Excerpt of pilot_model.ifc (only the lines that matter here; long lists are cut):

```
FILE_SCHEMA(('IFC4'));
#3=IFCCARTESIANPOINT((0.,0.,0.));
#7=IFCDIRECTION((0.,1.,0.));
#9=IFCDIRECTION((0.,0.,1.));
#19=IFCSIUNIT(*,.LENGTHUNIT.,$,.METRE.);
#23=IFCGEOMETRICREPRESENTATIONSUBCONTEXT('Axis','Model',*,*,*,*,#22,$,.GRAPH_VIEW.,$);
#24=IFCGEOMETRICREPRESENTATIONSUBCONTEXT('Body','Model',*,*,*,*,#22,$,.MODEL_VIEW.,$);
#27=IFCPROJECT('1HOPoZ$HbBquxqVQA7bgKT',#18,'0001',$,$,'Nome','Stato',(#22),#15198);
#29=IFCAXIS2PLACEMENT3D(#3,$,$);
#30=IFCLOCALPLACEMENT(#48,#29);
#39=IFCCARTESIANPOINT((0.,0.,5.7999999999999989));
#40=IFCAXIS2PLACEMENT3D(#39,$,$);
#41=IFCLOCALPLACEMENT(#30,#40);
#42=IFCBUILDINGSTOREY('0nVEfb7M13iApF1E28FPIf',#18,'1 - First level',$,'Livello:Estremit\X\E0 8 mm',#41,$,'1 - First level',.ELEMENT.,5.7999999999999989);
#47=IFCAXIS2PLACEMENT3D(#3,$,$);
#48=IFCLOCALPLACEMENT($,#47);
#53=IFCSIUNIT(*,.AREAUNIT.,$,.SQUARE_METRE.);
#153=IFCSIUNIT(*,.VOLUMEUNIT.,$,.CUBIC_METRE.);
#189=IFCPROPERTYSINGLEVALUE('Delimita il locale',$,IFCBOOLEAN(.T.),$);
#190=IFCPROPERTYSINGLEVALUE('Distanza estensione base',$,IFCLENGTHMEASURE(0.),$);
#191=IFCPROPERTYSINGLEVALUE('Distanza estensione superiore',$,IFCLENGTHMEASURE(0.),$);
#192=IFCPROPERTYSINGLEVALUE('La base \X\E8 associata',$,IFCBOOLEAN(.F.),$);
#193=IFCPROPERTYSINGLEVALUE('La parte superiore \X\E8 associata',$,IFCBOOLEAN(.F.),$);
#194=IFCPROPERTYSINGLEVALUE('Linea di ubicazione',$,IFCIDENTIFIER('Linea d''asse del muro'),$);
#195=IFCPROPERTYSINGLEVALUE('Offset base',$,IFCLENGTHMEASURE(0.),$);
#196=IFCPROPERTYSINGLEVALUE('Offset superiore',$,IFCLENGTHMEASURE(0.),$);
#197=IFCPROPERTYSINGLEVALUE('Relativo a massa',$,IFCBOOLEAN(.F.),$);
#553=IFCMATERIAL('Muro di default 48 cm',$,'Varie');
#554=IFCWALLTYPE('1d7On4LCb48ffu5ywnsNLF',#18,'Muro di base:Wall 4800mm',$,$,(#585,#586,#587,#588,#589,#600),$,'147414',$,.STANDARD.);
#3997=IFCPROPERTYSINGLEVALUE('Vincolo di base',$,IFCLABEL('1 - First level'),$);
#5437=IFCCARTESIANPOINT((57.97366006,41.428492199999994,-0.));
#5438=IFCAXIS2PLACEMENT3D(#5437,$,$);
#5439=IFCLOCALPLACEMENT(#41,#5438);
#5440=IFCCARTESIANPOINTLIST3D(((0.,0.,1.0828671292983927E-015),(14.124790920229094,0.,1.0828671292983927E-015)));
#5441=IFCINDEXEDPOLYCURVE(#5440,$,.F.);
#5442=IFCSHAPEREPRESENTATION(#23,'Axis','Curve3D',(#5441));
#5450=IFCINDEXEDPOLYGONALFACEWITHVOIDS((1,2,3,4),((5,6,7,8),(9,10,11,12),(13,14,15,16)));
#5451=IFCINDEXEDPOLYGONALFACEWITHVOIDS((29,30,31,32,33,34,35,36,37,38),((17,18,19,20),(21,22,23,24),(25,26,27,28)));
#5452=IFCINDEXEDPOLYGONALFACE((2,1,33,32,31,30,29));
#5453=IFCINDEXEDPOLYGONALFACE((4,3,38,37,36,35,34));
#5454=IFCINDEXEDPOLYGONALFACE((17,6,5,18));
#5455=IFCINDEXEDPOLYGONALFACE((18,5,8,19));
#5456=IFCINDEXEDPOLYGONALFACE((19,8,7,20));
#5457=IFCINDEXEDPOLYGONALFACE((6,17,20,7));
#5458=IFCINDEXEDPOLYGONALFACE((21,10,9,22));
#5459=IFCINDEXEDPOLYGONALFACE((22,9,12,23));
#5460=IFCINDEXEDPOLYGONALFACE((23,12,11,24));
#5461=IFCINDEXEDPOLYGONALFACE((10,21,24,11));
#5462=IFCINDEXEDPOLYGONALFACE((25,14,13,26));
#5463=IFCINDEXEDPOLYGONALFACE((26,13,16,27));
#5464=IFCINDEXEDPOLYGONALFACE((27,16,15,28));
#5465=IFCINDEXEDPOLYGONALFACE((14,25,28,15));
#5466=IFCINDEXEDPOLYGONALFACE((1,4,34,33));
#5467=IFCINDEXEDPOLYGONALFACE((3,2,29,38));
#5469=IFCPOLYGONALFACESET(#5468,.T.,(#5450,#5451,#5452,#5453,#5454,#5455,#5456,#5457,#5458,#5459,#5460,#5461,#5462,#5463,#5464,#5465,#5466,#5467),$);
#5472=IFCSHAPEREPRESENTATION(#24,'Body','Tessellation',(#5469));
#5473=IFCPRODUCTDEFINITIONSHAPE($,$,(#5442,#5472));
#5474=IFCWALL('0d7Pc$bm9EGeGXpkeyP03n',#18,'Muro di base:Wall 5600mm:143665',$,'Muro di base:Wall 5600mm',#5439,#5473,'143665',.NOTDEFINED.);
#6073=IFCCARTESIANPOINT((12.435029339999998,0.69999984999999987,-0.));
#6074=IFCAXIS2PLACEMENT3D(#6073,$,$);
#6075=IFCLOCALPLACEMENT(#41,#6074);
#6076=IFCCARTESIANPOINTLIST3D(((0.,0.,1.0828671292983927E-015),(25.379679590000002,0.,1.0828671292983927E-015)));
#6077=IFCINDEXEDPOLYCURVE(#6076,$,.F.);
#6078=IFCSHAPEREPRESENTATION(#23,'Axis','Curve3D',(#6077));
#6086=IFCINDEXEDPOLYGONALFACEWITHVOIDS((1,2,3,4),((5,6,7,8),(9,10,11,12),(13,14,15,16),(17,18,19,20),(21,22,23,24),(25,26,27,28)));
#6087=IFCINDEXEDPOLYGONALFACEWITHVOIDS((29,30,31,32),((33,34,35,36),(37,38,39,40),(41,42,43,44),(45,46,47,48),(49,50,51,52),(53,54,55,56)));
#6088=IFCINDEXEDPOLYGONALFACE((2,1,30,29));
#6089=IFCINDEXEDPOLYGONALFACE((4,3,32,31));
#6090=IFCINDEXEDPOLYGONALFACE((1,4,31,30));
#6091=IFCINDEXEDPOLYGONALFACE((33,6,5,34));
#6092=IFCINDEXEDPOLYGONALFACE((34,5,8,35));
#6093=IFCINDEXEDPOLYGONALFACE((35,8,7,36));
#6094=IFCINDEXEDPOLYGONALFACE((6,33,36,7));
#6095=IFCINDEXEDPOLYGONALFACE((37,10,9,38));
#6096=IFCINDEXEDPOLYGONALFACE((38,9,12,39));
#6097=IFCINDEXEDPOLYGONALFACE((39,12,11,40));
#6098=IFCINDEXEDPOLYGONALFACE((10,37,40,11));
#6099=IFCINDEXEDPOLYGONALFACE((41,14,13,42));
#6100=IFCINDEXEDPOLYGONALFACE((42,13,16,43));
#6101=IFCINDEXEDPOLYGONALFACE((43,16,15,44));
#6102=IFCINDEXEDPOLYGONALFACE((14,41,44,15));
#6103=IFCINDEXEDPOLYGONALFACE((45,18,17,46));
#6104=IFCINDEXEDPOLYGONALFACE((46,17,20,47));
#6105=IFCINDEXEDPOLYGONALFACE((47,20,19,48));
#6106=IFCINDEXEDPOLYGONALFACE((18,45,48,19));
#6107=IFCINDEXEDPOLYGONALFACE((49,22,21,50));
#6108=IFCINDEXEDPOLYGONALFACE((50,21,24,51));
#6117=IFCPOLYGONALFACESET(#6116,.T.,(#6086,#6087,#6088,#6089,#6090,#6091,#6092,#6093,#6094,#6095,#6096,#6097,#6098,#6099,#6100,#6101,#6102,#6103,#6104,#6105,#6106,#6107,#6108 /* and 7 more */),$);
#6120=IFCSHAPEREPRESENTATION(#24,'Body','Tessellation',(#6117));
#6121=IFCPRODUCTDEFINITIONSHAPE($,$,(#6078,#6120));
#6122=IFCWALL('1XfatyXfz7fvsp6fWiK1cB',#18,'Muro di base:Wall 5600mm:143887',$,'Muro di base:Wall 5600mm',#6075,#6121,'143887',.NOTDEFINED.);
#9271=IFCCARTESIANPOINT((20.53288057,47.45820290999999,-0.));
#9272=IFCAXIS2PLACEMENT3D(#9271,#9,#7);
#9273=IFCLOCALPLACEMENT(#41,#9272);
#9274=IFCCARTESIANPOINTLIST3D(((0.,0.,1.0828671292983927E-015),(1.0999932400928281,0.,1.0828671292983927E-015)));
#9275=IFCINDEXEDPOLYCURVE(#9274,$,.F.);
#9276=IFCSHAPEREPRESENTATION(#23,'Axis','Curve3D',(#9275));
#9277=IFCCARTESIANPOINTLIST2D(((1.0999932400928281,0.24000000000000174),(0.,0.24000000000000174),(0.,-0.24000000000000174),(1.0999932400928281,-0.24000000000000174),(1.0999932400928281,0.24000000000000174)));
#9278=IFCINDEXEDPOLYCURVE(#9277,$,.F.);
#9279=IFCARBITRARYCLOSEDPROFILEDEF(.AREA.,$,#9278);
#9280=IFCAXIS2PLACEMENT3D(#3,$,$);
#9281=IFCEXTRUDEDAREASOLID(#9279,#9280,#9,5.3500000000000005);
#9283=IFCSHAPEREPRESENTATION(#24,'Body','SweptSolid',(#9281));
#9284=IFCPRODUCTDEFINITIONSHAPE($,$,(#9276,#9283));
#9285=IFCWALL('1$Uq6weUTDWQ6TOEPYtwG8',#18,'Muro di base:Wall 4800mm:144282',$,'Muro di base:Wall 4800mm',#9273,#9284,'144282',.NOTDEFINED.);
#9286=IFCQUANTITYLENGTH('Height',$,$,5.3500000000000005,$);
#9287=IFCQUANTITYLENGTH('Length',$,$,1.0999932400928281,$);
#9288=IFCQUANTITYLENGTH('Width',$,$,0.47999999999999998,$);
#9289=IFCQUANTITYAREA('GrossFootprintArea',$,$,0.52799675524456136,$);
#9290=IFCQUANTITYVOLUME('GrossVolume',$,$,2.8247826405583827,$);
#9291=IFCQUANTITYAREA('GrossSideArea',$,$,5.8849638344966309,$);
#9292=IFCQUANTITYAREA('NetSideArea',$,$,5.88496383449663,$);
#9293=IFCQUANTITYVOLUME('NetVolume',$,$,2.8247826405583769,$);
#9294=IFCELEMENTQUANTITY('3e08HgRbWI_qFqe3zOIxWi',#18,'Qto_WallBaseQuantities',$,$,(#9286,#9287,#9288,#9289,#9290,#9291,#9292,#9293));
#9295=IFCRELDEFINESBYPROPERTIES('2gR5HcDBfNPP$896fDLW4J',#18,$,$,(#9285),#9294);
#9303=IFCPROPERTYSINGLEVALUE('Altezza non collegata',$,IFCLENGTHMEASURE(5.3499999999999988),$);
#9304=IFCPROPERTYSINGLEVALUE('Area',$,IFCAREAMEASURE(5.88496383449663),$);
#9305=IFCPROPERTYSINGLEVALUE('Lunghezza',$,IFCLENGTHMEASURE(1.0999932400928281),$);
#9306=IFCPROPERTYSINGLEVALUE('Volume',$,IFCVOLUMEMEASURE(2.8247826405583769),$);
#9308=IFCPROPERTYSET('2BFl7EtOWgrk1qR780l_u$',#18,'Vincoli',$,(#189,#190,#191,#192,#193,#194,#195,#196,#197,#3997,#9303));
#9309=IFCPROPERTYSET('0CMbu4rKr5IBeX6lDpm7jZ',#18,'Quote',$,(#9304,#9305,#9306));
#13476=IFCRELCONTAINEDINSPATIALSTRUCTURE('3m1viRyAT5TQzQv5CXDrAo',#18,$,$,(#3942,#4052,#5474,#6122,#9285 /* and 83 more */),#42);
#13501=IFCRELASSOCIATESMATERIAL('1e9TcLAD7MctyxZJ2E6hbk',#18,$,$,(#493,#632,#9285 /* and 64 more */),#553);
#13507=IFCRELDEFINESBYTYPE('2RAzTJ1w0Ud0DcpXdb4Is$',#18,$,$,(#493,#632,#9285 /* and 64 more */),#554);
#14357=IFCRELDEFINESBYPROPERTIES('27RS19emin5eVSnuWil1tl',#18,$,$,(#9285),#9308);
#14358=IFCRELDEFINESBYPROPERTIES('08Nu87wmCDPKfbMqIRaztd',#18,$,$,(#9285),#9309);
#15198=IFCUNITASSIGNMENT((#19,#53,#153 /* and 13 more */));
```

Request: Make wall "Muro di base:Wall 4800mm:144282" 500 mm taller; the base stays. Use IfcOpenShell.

```python
import ifcopenshell
import ifcopenshell.api.pset
import ifcopenshell.geom
import ifcopenshell.util.element
import ifcopenshell.util.representation
import ifcopenshell.util.shape
import ifcopenshell.util.unit

model = ifcopenshell.open("pilot_model.ifc")
unit_scale = ifcopenshell.util.unit.calculate_unit_scale(model)
area_scale = ifcopenshell.util.unit.calculate_unit_scale(model, "AREAUNIT")
volume_scale = ifcopenshell.util.unit.calculate_unit_scale(model, "VOLUMEUNIT")
settings = ifcopenshell.geom.settings()


def volume(element):
    """Net volume in cubic metres, openings subtracted."""
    shape = ifcopenshell.geom.create_shape(settings, element)
    return ifcopenshell.util.shape.get_volume(shape.geometry)


wall = model.by_guid("1$Uq6weUTDWQ6TOEPYtwG8")
before = volume(wall)

body = ifcopenshell.util.representation.get_representation(wall, "Model", "Body")
solid = body.Items[0]
old_height = solid.Depth
solid.Depth += 0.5 / unit_scale
after = volume(wall)
thickness = 0.48  # wall thickness in metres

# Update the stored height, areas and volumes.
qto = model.by_id(ifcopenshell.util.element.get_pset(wall, "Qto_WallBaseQuantities", should_inherit=False)["id"])
ifcopenshell.api.pset.edit_qto(model, qto=qto, properties={
    "Height": solid.Depth,
    "GrossVolume": ifcopenshell.util.element.get_pset(wall, "Qto_WallBaseQuantities", "GrossVolume") * solid.Depth / old_height,
    "GrossSideArea": ifcopenshell.util.element.get_pset(wall, "Qto_WallBaseQuantities", "GrossSideArea") * solid.Depth / old_height,
    "NetSideArea": after / thickness / area_scale,
    "NetVolume": after / volume_scale,
})
pset = model.by_id(ifcopenshell.util.element.get_pset(wall, "Vincoli", should_inherit=False)["id"])
ifcopenshell.api.pset.edit_pset(model, pset=pset, properties={
    "Altezza non collegata": model.create_entity("IfcLengthMeasure", solid.Depth),
})
pset = model.by_id(ifcopenshell.util.element.get_pset(wall, "Quote", should_inherit=False)["id"])
ifcopenshell.api.pset.edit_pset(model, pset=pset, properties={
    "Area": model.create_entity("IfcAreaMeasure", after / thickness / area_scale),
    "Volume": model.create_entity("IfcVolumeMeasure", after / volume_scale),
})

print(f"height {old_height:g} -> {solid.Depth:g}, volume {before:.3f} -> {after:.3f} m3")

model.write("pilot_model_edited.ifc")
```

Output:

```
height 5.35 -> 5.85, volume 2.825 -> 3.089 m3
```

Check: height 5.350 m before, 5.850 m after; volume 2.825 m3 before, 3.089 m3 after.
